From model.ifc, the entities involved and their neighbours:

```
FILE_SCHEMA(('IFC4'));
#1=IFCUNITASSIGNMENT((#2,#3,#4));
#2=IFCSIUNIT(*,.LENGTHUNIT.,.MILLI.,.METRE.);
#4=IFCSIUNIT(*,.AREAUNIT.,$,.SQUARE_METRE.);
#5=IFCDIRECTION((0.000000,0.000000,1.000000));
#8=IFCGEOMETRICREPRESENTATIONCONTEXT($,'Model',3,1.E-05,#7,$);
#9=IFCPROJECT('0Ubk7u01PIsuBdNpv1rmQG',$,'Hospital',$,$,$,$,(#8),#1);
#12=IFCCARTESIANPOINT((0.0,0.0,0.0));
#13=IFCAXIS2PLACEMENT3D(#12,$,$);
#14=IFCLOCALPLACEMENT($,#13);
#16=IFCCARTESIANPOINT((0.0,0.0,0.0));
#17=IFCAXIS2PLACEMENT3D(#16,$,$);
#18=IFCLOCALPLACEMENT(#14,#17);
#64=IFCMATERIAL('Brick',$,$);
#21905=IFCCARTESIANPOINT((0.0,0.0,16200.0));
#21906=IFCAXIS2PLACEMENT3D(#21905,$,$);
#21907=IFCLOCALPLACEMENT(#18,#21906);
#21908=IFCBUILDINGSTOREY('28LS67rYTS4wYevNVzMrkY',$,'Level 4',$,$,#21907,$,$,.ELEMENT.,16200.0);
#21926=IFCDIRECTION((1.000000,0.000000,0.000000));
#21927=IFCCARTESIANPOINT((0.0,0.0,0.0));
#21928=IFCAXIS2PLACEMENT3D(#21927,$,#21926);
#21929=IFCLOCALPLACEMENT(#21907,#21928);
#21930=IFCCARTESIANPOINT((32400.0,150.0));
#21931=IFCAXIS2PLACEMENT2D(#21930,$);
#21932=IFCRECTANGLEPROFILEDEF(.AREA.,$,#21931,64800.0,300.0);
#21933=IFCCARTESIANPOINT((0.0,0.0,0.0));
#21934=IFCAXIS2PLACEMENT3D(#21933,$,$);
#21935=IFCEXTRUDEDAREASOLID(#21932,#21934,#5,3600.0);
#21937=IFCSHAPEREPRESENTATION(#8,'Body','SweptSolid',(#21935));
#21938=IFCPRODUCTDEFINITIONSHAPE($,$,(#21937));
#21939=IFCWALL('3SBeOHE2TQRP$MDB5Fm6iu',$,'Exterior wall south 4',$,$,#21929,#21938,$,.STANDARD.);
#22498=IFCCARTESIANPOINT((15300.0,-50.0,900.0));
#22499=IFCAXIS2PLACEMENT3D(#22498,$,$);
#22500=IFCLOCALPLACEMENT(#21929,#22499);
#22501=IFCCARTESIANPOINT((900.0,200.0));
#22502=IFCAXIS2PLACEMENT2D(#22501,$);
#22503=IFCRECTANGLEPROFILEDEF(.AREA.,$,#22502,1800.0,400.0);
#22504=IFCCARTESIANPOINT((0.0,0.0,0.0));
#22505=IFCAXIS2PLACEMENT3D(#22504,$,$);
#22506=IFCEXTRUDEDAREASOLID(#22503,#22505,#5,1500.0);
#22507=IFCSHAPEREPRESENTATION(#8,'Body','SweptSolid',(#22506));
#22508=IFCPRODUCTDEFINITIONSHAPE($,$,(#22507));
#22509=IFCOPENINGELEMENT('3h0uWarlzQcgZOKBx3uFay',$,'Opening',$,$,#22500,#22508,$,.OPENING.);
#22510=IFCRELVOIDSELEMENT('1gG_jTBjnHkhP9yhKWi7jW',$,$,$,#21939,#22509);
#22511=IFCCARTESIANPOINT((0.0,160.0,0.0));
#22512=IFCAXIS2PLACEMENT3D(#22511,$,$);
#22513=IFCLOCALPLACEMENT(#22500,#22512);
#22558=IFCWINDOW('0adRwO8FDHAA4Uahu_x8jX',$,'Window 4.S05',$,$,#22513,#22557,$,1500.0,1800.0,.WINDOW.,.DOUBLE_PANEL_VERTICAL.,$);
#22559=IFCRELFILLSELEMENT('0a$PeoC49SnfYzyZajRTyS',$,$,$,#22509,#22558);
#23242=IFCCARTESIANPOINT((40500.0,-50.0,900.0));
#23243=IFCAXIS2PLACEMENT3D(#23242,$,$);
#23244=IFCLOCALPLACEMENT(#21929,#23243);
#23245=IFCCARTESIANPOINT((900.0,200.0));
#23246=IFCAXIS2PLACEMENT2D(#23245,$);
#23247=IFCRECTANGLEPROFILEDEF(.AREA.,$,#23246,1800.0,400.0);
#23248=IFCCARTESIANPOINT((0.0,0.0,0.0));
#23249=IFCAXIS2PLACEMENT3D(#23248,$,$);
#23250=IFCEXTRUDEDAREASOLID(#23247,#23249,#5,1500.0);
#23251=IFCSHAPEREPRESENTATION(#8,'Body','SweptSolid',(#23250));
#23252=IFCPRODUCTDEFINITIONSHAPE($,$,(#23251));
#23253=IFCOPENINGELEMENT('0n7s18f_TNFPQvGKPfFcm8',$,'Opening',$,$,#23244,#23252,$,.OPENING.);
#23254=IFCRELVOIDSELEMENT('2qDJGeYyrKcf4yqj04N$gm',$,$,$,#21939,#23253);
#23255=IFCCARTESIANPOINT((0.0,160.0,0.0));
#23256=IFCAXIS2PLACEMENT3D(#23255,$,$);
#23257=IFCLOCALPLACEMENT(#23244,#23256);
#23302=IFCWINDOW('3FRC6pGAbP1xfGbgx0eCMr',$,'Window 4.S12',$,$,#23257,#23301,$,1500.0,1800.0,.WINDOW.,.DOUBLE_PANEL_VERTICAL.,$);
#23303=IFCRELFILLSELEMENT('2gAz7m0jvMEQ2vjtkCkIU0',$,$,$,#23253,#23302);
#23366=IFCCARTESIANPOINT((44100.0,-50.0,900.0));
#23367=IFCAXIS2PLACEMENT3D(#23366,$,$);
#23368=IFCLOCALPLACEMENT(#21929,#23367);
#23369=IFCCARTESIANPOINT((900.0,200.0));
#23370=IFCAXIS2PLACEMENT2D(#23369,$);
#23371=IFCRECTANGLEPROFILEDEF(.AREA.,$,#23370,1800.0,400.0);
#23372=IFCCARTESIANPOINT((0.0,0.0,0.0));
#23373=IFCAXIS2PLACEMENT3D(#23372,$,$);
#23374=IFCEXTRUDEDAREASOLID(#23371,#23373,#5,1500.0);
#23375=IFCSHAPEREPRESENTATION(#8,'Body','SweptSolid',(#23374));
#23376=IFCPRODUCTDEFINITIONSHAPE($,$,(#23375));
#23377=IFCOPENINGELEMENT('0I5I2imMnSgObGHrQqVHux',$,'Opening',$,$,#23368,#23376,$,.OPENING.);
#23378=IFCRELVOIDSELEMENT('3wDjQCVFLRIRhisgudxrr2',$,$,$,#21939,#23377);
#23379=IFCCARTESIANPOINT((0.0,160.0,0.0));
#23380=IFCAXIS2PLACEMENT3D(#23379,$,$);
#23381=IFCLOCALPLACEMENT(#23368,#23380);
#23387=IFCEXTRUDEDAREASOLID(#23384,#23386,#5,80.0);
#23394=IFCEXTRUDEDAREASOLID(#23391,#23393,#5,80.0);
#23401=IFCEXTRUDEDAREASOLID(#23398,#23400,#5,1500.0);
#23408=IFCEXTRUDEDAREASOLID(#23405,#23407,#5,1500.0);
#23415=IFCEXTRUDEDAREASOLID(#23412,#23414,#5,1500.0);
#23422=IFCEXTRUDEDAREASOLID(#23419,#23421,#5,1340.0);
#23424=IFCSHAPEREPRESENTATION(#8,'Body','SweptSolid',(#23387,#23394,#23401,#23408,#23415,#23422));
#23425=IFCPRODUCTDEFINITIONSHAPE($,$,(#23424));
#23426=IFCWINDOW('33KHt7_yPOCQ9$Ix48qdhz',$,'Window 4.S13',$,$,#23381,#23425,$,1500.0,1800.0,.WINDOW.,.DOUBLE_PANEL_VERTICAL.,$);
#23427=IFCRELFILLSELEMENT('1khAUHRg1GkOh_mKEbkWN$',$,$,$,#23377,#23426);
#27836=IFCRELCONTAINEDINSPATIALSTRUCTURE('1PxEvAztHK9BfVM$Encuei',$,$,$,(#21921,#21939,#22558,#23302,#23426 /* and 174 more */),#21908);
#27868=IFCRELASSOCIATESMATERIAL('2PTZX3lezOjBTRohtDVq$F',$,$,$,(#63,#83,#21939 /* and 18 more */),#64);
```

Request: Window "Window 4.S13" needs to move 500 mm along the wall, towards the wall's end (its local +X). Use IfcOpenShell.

```python
import ifcopenshell
import ifcopenshell.api.geometry
import ifcopenshell.util.placement
import ifcopenshell.util.unit

model = ifcopenshell.open("model.ifc")
unit_scale = ifcopenshell.util.unit.calculate_unit_scale(model)

window = model.by_guid("33KHt7_yPOCQ9$Ix48qdhz")
opening = window.FillsVoids[0].RelatingOpeningElement
wall = opening.VoidsElements[0].RelatingBuildingElement

wall_matrix = ifcopenshell.util.placement.get_local_placement(wall.ObjectPlacement)
shift = wall_matrix[:3, 0] * 0.5 / unit_scale
before = ifcopenshell.util.placement.get_local_placement(window.ObjectPlacement)[:3, 3].copy()

# The window is placed relative to its opening, so it follows when the opening moves.
matrix = ifcopenshell.util.placement.get_local_placement(opening.ObjectPlacement)
matrix[:3, 3] += shift
ifcopenshell.api.geometry.edit_object_placement(
    model, product=opening, matrix=matrix, is_si=False, should_transform_children=True
)

after = ifcopenshell.util.placement.get_local_placement(window.ObjectPlacement)[:3, 3]
print("window moved by", (after - before).round(3) + 0.0)

model.write("model_rev.ifc")
```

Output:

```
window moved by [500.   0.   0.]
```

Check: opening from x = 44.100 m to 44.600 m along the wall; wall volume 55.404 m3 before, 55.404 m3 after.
